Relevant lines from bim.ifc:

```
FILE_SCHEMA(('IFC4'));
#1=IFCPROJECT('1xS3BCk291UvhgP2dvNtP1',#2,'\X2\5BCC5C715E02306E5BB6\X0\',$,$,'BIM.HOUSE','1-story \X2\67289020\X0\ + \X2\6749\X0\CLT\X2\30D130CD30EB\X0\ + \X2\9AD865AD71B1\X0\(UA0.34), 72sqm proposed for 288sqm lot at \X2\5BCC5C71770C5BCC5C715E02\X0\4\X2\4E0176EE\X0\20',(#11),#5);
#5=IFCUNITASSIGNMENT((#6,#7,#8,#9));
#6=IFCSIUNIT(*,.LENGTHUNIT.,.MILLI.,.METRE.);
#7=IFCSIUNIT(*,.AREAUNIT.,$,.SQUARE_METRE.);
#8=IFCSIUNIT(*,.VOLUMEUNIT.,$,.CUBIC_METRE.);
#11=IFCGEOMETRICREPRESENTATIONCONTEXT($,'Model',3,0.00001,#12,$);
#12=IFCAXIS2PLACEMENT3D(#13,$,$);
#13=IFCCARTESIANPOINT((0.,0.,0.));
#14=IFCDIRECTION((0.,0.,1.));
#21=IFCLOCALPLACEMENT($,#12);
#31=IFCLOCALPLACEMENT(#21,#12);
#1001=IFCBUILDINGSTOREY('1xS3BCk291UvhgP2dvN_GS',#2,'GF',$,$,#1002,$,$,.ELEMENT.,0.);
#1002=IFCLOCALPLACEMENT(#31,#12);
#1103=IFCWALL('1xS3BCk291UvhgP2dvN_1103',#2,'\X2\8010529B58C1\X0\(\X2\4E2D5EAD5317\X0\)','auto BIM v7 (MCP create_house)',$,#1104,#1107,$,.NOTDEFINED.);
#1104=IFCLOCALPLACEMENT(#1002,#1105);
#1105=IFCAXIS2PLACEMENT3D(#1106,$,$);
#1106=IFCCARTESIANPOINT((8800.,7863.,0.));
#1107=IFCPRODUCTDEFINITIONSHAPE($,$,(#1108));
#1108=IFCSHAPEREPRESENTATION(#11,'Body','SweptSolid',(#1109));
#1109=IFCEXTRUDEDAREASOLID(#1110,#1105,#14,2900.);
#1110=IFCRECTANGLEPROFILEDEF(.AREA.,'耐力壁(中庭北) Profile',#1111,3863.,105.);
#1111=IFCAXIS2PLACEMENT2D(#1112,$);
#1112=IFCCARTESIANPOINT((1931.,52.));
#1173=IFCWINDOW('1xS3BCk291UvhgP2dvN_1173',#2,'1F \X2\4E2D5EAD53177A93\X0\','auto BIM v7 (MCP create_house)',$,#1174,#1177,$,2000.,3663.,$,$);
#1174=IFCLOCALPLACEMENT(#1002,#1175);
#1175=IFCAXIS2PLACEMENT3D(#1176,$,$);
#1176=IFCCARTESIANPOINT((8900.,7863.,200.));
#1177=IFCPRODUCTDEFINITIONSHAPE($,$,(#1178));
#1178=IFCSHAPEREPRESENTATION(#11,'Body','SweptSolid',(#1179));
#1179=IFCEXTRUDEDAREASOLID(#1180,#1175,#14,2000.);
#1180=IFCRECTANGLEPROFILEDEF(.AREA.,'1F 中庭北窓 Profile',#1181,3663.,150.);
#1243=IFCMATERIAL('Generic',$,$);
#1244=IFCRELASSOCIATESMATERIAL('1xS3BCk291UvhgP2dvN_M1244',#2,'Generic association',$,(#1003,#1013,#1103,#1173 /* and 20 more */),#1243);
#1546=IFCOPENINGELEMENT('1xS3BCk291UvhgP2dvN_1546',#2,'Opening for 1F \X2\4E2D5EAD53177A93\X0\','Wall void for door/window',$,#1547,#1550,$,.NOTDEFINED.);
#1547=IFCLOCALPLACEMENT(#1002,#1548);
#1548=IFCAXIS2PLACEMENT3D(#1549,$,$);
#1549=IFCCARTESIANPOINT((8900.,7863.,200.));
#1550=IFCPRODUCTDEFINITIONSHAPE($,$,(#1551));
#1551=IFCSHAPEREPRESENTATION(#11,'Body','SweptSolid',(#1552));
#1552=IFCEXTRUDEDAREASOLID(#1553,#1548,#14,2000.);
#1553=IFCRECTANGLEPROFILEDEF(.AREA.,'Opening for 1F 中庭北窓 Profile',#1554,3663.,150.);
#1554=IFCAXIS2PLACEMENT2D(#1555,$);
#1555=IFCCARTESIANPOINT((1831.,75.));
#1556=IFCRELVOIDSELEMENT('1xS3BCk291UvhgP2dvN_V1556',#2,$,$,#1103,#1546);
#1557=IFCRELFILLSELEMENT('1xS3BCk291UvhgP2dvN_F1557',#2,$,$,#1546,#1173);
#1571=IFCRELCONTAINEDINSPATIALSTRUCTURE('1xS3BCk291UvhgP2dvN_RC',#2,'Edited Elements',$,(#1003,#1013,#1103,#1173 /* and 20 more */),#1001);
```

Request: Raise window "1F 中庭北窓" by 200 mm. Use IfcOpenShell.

```python
import numpy as np
import ifcopenshell
import ifcopenshell.api.geometry
import ifcopenshell.util.placement
import ifcopenshell.util.unit

model = ifcopenshell.open("bim.ifc")
unit_scale = ifcopenshell.util.unit.calculate_unit_scale(model)

window = model.by_id(1173)
opening = window.FillsVoids[0].RelatingOpeningElement
dz = 0.2 / unit_scale

shift = np.array([0.0, 0.0, dz])
# The window is not placed relative to its opening, so move both.
for product in (opening, window):
    matrix = ifcopenshell.util.placement.get_local_placement(product.ObjectPlacement)
    matrix[:3, 3] += shift
    ifcopenshell.api.geometry.edit_object_placement(model, product=product, matrix=matrix, is_si=False)

print(f"moved by {dz * unit_scale:+.3f} m")

model.write("bim_edited.ifc")
```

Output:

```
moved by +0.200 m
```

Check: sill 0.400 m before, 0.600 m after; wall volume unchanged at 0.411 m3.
